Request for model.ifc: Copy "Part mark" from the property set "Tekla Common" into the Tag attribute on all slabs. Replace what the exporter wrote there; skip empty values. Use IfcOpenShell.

First a look at what the model holds.

```python
import ifcopenshell
import ifcopenshell.util.element

model = ifcopenshell.open("model.ifc")
print(model.schema)
slabs = model.by_type("IfcSlab")
print(len(slabs), "slabs")
for e in slabs[:8]:
    source = ifcopenshell.util.element.get_pset(e, "Tekla Common", "Part mark")
    target = e.Tag
    print(e.id(), repr(source), repr(target), sep=" | ")
```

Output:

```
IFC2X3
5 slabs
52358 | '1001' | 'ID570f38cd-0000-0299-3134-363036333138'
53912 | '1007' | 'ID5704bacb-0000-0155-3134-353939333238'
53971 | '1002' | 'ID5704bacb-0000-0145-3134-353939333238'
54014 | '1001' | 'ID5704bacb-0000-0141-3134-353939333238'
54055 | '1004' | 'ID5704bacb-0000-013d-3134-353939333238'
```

```python
import ifcopenshell
import ifcopenshell.util.element

model = ifcopenshell.open("model.ifc")

count = 0
for e in model.by_type("IfcSlab"):
    value = ifcopenshell.util.element.get_pset(e, "Tekla Common", "Part mark")
    current = e.Tag
    if not value or not value.strip() or current == value:
        continue
    e.Tag = value
    count += 1

print(count, "slabs updated")

model.write("model_v2.ifc")
```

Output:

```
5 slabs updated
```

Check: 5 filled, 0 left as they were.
